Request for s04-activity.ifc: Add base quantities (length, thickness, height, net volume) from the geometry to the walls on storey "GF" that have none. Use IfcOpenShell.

First a look at what the model holds.

```python
import ifcopenshell
import ifcopenshell.util.element
import ifcopenshell.util.unit

model = ifcopenshell.open("s04-activity.ifc")
print(model.schema)
for unit_type in ("LENGTHUNIT", "AREAUNIT", "VOLUMEUNIT"):
    print(unit_type, ifcopenshell.util.unit.calculate_unit_scale(model, unit_type))
storey = next(s for s in model.by_type("IfcBuildingStorey") if s.Name == "GF")
walls = [e for e in ifcopenshell.util.element.get_decomposition(storey) if e.is_a("IfcWall")]
for e in sorted(walls, key=lambda e: e.id()):
    print(e.id(), e.is_a(), e.Name, list(ifcopenshell.util.element.get_psets(e, qtos_only=True)), sep=" | ")
```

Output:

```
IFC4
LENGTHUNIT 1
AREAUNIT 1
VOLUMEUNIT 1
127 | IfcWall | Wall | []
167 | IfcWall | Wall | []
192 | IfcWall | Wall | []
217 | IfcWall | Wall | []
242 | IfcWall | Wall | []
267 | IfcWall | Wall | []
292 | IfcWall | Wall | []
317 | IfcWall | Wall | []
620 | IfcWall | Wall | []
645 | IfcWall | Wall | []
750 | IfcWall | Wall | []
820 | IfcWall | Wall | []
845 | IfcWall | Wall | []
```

```python
import ifcopenshell
import ifcopenshell.api.pset
import ifcopenshell.geom
import ifcopenshell.util.element
import ifcopenshell.util.shape
import ifcopenshell.util.unit

model = ifcopenshell.open("s04-activity.ifc")
unit_scale = ifcopenshell.util.unit.calculate_unit_scale(model)
volume_scale = ifcopenshell.util.unit.calculate_unit_scale(model, "VOLUMEUNIT")
settings = ifcopenshell.geom.settings()

storey = next(s for s in model.by_type("IfcBuildingStorey") if s.Name == "GF")
walls = [e for e in ifcopenshell.util.element.get_decomposition(storey) if e.is_a("IfcWall")]

for e in sorted(walls, key=lambda e: e.id()):
    if ifcopenshell.util.element.get_psets(e, qtos_only=True, should_inherit=False):
        continue
    # Geometry comes back in metres, in the element's own axes.
    shape = ifcopenshell.geom.create_shape(settings, e)
    values = {
        "Length": ifcopenshell.util.shape.get_x(shape.geometry) / unit_scale,
        "Width": ifcopenshell.util.shape.get_y(shape.geometry) / unit_scale,
        "Height": ifcopenshell.util.shape.get_z(shape.geometry) / unit_scale,
        "NetVolume": ifcopenshell.util.shape.get_volume(shape.geometry) / volume_scale,
    }
    qto = ifcopenshell.api.pset.add_qto(model, product=e, name="Qto_WallBaseQuantities")
    ifcopenshell.api.pset.edit_qto(model, qto=qto, properties=values)
    print(e.id(), {k: round(v, 3) for k, v in values.items()})

model.write("s04-activity_updated.ifc")
```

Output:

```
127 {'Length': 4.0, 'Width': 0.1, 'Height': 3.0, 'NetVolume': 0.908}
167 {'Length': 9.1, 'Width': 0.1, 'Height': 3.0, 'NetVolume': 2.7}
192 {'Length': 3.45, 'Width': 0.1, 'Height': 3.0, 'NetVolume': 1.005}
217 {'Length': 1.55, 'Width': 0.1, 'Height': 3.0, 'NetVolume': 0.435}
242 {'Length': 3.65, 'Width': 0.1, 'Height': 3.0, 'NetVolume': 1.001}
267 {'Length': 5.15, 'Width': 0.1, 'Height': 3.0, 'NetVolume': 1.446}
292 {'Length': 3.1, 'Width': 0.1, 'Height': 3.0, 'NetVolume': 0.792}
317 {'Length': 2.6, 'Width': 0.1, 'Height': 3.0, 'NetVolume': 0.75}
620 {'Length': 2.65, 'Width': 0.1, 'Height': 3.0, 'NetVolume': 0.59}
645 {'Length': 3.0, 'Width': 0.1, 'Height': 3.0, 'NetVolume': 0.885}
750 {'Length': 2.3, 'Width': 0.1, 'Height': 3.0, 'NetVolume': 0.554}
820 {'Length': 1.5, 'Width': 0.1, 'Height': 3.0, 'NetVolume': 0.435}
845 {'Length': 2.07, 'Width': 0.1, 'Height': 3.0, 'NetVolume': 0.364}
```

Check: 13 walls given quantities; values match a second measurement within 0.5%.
